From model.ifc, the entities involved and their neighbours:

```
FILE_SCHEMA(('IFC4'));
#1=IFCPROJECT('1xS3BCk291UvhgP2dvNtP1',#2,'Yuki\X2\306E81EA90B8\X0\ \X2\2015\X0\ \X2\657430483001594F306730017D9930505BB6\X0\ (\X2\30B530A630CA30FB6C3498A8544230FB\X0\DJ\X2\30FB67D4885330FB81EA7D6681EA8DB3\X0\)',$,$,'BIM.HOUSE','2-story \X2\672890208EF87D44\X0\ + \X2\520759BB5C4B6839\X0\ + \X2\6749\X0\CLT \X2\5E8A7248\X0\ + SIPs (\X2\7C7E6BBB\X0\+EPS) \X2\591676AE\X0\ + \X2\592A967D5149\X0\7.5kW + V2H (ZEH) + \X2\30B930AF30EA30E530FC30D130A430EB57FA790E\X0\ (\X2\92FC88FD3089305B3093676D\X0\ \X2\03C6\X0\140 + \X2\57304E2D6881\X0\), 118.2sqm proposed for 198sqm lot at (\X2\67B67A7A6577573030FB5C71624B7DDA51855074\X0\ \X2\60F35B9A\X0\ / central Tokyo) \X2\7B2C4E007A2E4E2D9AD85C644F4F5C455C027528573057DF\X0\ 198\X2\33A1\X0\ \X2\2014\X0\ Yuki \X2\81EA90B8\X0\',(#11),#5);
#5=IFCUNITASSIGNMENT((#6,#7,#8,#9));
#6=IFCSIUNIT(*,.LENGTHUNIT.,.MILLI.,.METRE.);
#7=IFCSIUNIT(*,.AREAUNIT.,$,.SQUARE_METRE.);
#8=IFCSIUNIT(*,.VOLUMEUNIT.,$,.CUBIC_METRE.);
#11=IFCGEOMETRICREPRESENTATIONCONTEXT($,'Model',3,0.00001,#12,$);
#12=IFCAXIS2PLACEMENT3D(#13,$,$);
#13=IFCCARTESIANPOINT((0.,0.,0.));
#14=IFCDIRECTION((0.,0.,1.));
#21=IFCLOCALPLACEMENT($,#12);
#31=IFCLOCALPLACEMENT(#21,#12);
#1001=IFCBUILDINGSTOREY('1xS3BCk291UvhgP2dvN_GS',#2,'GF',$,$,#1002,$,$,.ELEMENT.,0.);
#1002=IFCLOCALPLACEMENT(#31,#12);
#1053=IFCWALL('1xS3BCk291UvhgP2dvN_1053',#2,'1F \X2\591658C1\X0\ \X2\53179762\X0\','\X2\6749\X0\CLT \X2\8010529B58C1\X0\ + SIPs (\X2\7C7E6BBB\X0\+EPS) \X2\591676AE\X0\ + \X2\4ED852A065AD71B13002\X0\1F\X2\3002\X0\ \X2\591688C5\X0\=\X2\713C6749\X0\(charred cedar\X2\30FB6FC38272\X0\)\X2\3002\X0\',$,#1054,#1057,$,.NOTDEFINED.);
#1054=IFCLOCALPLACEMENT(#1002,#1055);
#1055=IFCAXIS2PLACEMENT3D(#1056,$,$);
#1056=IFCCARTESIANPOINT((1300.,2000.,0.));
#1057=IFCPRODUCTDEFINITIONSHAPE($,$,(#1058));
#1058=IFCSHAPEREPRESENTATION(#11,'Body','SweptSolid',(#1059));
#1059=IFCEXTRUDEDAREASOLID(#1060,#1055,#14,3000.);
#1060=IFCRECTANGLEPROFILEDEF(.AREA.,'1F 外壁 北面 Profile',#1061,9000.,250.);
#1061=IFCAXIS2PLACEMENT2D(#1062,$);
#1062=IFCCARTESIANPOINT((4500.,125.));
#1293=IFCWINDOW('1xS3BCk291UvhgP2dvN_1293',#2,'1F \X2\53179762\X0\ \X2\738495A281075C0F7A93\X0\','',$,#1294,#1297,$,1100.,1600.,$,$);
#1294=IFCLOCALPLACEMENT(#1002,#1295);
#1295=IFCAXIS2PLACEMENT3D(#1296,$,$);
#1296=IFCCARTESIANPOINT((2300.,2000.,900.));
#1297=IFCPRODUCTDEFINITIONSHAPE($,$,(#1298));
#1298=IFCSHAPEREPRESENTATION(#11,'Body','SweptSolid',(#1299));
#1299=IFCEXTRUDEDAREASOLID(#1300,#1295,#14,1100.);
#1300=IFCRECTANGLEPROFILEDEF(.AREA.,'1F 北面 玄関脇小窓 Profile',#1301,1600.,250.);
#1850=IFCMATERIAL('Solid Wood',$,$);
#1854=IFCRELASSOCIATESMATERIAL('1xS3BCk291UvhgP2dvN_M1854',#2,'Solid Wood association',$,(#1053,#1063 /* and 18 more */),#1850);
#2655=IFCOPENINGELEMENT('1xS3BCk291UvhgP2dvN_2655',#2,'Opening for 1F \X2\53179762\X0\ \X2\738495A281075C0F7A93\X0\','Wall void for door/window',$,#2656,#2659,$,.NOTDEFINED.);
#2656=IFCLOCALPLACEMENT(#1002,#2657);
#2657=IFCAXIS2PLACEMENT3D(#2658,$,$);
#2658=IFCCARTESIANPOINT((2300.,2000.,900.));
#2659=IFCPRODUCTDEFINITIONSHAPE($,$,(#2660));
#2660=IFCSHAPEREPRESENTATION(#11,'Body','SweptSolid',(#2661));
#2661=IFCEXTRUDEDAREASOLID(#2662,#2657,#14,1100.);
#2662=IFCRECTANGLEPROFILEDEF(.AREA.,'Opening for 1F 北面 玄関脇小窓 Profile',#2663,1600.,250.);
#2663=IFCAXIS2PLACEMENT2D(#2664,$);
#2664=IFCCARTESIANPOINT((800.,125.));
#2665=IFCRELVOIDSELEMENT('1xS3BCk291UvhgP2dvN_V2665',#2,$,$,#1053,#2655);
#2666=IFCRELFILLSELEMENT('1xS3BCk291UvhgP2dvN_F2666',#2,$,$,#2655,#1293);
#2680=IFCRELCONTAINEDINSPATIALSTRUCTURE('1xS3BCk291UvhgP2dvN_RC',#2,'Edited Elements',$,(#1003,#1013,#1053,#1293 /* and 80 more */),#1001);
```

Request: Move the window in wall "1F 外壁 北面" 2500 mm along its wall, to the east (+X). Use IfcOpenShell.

```python
import ifcopenshell
import ifcopenshell.api.geometry
import ifcopenshell.util.placement

model = ifcopenshell.open("model.ifc")

window = model.by_id(1293)
opening = window.FillsVoids[0].RelatingOpeningElement
wall = opening.VoidsElements[0].RelatingBuildingElement

wall_matrix = ifcopenshell.util.placement.get_local_placement(wall.ObjectPlacement)
shift = wall_matrix[:3, 0] * 2500.0
before = ifcopenshell.util.placement.get_local_placement(window.ObjectPlacement)[:3, 3].copy()

# The window is not placed relative to its opening, so move both.
for product in (opening, window):
    matrix = ifcopenshell.util.placement.get_local_placement(product.ObjectPlacement)
    matrix[:3, 3] += shift
    ifcopenshell.api.geometry.edit_object_placement(model, product=product, matrix=matrix, is_si=False)

after = ifcopenshell.util.placement.get_local_placement(window.ObjectPlacement)[:3, 3]
print("window moved by", (after - before).round(3) + 0.0)

model.write("model_v2.ifc")
```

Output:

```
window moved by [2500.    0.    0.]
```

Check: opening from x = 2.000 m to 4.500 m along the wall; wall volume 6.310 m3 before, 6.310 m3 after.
